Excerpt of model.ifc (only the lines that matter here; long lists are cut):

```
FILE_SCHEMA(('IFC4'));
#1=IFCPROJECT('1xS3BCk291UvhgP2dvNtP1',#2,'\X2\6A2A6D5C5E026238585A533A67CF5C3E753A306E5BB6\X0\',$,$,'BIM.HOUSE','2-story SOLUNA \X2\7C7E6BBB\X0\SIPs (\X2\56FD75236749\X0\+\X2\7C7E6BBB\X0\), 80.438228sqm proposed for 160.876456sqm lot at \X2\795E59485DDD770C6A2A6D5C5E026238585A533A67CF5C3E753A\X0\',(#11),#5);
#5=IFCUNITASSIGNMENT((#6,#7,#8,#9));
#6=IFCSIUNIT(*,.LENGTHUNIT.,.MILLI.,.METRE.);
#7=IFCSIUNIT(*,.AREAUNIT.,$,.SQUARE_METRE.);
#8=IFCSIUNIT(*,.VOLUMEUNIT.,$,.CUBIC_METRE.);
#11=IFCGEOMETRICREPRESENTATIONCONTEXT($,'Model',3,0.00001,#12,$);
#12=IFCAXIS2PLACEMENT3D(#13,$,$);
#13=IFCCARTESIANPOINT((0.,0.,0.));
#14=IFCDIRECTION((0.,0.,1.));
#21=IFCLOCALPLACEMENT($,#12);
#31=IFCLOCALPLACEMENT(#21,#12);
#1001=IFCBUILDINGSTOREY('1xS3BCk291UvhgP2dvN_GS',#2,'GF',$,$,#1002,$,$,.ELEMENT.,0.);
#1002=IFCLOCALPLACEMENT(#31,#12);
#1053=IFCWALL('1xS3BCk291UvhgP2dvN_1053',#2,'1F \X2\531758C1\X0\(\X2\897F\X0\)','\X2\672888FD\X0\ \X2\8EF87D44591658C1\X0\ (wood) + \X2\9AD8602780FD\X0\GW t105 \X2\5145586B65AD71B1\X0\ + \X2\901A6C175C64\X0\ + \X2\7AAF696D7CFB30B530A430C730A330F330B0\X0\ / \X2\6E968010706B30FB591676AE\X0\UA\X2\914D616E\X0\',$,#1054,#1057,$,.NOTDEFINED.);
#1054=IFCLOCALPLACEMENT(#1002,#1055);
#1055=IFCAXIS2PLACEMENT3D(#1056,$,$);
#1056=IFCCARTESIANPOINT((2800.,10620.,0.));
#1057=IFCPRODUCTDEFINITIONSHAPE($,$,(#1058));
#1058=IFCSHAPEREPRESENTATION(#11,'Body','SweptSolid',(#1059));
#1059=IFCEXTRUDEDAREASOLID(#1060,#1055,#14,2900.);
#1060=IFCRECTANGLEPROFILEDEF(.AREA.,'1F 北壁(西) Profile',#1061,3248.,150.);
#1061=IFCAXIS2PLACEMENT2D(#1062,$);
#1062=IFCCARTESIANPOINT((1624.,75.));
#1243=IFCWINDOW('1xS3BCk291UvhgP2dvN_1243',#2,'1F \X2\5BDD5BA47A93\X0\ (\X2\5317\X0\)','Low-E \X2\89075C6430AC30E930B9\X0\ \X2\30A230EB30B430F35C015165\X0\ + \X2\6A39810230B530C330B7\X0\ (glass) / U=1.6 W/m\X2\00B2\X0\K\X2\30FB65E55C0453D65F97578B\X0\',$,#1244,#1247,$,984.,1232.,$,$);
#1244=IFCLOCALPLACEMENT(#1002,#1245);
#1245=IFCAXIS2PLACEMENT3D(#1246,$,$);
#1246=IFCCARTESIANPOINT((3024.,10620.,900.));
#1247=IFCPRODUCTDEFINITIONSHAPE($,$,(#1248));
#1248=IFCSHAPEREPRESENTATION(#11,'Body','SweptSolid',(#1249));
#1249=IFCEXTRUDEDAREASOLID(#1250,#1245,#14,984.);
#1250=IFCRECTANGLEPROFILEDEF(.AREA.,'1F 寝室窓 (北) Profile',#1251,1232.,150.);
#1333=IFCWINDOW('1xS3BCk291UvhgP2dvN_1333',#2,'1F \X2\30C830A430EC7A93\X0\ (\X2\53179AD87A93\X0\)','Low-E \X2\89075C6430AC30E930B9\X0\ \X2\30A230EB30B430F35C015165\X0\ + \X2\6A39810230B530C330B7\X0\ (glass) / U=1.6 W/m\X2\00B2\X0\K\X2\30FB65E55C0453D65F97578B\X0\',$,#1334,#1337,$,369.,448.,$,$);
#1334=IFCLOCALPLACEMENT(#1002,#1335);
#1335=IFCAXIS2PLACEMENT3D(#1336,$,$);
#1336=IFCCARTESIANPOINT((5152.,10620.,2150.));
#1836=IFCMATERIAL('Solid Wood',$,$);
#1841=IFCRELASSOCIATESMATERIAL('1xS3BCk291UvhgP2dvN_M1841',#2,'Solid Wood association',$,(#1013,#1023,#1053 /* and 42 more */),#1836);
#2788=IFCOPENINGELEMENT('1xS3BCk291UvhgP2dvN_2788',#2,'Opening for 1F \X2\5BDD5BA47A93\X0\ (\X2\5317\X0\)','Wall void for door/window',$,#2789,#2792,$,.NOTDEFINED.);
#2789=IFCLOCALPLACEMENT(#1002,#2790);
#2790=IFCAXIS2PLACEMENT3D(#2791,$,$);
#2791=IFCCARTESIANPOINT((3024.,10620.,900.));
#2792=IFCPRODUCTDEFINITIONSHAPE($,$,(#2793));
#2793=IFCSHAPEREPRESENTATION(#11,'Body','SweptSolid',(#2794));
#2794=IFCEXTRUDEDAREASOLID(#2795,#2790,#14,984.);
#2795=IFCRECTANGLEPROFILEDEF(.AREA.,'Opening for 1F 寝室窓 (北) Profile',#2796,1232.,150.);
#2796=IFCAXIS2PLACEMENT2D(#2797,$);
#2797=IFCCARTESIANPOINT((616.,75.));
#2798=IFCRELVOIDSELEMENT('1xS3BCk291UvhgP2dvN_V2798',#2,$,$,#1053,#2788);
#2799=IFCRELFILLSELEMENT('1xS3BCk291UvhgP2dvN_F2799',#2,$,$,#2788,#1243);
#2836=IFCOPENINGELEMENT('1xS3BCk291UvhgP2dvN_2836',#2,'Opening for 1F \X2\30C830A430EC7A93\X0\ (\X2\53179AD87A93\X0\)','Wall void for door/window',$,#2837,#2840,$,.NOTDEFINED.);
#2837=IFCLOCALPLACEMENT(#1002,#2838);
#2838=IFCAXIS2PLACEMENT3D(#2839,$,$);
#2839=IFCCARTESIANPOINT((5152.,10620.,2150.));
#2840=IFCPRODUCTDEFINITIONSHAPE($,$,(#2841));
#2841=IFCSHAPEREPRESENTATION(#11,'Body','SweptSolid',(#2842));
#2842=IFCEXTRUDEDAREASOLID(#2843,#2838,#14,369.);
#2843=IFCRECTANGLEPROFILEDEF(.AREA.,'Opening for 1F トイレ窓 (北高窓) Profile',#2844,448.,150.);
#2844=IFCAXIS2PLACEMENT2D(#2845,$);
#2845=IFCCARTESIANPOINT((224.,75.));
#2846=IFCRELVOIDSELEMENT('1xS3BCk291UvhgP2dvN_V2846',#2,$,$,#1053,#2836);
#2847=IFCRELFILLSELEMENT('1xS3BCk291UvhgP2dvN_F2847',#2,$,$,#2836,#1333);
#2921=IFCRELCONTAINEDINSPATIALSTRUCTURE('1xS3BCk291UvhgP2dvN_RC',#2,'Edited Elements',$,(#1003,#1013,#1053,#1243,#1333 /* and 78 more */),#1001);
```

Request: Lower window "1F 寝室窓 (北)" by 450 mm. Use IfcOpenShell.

```python
import numpy as np
import ifcopenshell
import ifcopenshell.api.geometry
import ifcopenshell.util.placement
import ifcopenshell.util.unit

model = ifcopenshell.open("model.ifc")
unit_scale = ifcopenshell.util.unit.calculate_unit_scale(model)

window = model.by_guid("1xS3BCk291UvhgP2dvN_1243")
opening = window.FillsVoids[0].RelatingOpeningElement
dz = -0.45 / unit_scale

shift = np.array([0.0, 0.0, dz])
# The window is not placed relative to its opening, so move both.
for product in (opening, window):
    matrix = ifcopenshell.util.placement.get_local_placement(product.ObjectPlacement)
    matrix[:3, 3] += shift
    ifcopenshell.api.geometry.edit_object_placement(model, product=product, matrix=matrix, is_si=False)

print(f"moved by {dz * unit_scale:+.3f} m")

model.write("model-out.ifc")
```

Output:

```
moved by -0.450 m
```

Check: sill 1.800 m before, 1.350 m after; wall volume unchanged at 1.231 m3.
